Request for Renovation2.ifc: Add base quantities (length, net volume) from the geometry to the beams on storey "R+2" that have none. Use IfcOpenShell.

First a look at what the model holds.

```python
import ifcopenshell
import ifcopenshell.util.element
import ifcopenshell.util.unit

model = ifcopenshell.open("Renovation2.ifc")
print(model.schema)
for unit_type in ("LENGTHUNIT", "AREAUNIT", "VOLUMEUNIT"):
    print(unit_type, ifcopenshell.util.unit.calculate_unit_scale(model, unit_type))
storey = next(s for s in model.by_type("IfcBuildingStorey") if s.Name == "R+2")
beams = [e for e in ifcopenshell.util.element.get_decomposition(storey) if e.is_a("IfcBeam")]
for e in sorted(beams, key=lambda e: e.id()):
    print(e.id(), e.is_a(), e.Name, list(ifcopenshell.util.element.get_psets(e, qtos_only=True)), sep=" | ")
```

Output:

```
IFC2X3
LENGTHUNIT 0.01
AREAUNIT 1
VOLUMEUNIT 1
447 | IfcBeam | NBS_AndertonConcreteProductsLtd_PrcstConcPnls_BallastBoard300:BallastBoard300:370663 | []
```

```python
import ifcopenshell
import ifcopenshell.api.pset
import ifcopenshell.geom
import ifcopenshell.util.element
import ifcopenshell.util.shape
import ifcopenshell.util.unit

model = ifcopenshell.open("Renovation2.ifc")
unit_scale = ifcopenshell.util.unit.calculate_unit_scale(model)
volume_scale = ifcopenshell.util.unit.calculate_unit_scale(model, "VOLUMEUNIT")
settings = ifcopenshell.geom.settings()

storey = next(s for s in model.by_type("IfcBuildingStorey") if s.Name == "R+2")
beams = [e for e in ifcopenshell.util.element.get_decomposition(storey) if e.is_a("IfcBeam")]

for e in sorted(beams, key=lambda e: e.id()):
    if ifcopenshell.util.element.get_psets(e, qtos_only=True, should_inherit=False):
        continue
    # Geometry comes back in metres, in the element's own axes.
    shape = ifcopenshell.geom.create_shape(settings, e)
    values = {
        "Length": ifcopenshell.util.shape.get_max_xyz(shape.geometry) / unit_scale,
        "NetVolume": ifcopenshell.util.shape.get_volume(shape.geometry) / volume_scale,
    }
    qto = ifcopenshell.api.pset.add_qto(model, product=e, name="BaseQuantities")
    ifcopenshell.api.pset.edit_qto(model, qto=qto, properties=values)
    print(e.id(), {k: round(v, 3) for k, v in values.items()})

model.write("Renovation2_updated.ifc")
```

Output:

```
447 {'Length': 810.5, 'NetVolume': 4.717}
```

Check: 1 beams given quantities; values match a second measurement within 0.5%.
